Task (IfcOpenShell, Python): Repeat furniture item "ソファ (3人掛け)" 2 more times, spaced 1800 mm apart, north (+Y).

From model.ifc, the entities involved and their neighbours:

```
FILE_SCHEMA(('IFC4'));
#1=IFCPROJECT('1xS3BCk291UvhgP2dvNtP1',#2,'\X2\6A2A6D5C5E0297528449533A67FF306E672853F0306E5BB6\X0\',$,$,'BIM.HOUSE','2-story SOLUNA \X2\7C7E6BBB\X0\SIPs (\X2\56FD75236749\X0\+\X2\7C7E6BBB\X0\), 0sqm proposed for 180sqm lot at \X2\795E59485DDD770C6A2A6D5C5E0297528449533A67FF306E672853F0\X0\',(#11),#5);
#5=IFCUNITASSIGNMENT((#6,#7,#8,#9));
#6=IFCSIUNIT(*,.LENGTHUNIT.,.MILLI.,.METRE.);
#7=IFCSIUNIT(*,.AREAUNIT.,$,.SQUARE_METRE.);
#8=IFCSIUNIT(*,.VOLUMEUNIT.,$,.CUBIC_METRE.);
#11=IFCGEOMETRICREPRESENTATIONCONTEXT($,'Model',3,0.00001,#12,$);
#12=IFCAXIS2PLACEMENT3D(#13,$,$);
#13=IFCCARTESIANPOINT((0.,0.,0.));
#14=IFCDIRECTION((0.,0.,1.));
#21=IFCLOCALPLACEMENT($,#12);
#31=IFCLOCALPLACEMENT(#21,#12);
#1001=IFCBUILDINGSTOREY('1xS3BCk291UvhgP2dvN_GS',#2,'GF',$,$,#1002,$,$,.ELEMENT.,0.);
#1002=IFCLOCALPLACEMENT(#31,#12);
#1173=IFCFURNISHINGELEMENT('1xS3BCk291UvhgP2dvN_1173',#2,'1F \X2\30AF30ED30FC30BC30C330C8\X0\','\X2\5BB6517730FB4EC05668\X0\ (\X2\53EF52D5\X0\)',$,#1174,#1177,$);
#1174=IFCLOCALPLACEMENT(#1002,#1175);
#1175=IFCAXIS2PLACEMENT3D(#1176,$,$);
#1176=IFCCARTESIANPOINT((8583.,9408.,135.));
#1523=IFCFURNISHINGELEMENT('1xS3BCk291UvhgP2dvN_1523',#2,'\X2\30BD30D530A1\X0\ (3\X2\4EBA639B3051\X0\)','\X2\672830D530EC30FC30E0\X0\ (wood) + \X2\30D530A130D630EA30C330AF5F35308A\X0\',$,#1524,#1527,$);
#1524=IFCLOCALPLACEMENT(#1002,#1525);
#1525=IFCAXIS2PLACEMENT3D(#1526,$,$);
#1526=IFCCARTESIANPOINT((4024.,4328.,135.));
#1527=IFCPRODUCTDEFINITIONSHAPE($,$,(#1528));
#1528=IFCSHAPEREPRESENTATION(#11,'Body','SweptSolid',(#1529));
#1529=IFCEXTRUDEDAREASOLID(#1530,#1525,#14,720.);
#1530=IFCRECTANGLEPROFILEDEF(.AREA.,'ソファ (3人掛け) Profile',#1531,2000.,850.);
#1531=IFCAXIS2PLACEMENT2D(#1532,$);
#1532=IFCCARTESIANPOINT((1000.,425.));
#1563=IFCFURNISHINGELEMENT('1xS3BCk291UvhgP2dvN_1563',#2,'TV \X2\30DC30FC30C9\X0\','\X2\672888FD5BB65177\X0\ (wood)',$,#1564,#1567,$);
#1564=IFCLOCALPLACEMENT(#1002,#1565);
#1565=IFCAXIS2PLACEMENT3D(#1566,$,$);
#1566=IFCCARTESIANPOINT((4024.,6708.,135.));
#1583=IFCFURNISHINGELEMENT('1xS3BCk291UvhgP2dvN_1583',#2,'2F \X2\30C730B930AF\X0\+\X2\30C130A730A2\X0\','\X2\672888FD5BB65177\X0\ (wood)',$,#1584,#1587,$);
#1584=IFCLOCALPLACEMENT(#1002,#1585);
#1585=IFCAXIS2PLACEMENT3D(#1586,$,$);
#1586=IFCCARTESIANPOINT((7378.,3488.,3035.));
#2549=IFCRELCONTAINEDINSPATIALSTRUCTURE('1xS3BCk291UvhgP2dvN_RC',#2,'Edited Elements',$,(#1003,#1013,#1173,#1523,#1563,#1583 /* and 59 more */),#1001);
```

```python
import numpy as np
import ifcopenshell
import ifcopenshell.api.geometry
import ifcopenshell.api.root
import ifcopenshell.util.element
import ifcopenshell.util.placement
import ifcopenshell.util.unit

model = ifcopenshell.open("model.ifc")
unit_scale = ifcopenshell.util.unit.calculate_unit_scale(model)


def reuse_history(source, copy):
    """copy_class also copies each property set's owner history, people and application; keep the originals."""
    for rel in copy.IsDefinedBy:
        if rel.is_a("IfcRelDefinesByProperties") and (history := rel.RelatingPropertyDefinition.OwnerHistory):
            rel.RelatingPropertyDefinition.OwnerHistory = source.OwnerHistory
            ifcopenshell.util.element.remove_deep2(model, history)


source = model.by_guid("1xS3BCk291UvhgP2dvN_1523")
base = ifcopenshell.util.placement.get_local_placement(source.ObjectPlacement)
step = np.array([0.0, 1.0, 0.0]) * 1.8 / unit_scale

for i in range(1, 3):
    copy = ifcopenshell.api.root.copy_class(model, product=source)
    copy.Representation = ifcopenshell.util.element.copy_deep(
        model, source.Representation, exclude=["IfcGeometricRepresentationContext", "IfcRepresentationMap"]
    )
    reuse_history(source, copy)
    matrix = base.copy()
    matrix[:3, 3] += i * step
    print("added at", matrix[:3, 3].round(3) + 0.0)
    ifcopenshell.api.geometry.edit_object_placement(model, product=copy, matrix=matrix, is_si=False)

model.write("model_v2.ifc")
```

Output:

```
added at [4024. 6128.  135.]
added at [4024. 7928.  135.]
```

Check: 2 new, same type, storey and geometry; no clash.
